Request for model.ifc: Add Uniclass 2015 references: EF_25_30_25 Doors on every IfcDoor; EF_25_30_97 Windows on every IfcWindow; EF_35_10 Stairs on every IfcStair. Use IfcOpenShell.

First a look at what the model holds.

```python
import ifcopenshell

model = ifcopenshell.open("model.ifc")
print(model.schema)
print("classifications:", [c.Name for c in model.by_type("IfcClassification")])
for ifc_class in ("IfcDoor", "IfcRoof", "IfcStair", "IfcWall", "IfcWindow"):
    print(ifc_class, len(model.by_type(ifc_class)))
```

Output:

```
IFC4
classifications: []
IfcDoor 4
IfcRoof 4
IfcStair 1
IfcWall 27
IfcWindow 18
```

```python
import ifcopenshell
import ifcopenshell.api.classification

model = ifcopenshell.open("model.ifc")

system = ifcopenshell.api.classification.add_classification(model, classification="Uniclass 2015")

codes = {
    "IfcDoor": ("EF_25_30_25", "Doors"),
    "IfcWindow": ("EF_25_30_97", "Windows"),
    "IfcStair": ("EF_35_10", "Stairs"),
}
for ifc_class, (code, name) in codes.items():
    products = model.by_type(ifc_class)
    ifcopenshell.api.classification.add_reference(
        model, products=products, classification=system, identification=code, name=name
    )
    print(code, len(products))

model.write("model_updated.ifc")
```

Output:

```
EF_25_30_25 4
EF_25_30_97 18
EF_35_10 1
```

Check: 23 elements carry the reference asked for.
